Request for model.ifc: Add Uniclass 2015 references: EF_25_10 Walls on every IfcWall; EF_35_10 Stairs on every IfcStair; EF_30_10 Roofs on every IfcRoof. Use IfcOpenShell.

First a look at what the model holds.

```python
import ifcopenshell

model = ifcopenshell.open("model.ifc")
print(model.schema)
print("classifications:", [c.Name for c in model.by_type("IfcClassification")])
for ifc_class in ("IfcDoor", "IfcRoof", "IfcStair", "IfcWall", "IfcWindow"):
    print(ifc_class, len(model.by_type(ifc_class)))
```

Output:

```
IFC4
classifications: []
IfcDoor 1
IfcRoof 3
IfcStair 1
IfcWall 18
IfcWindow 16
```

```python
import ifcopenshell
import ifcopenshell.api.classification

model = ifcopenshell.open("model.ifc")

system = ifcopenshell.api.classification.add_classification(model, classification="Uniclass 2015")

codes = {
    "IfcWall": ("EF_25_10", "Walls"),
    "IfcStair": ("EF_35_10", "Stairs"),
    "IfcRoof": ("EF_30_10", "Roofs"),
}
for ifc_class, (code, name) in codes.items():
    products = model.by_type(ifc_class)
    ifcopenshell.api.classification.add_reference(
        model, products=products, classification=system, identification=code, name=name
    )
    print(code, len(products))

model.write("model_updated.ifc")
```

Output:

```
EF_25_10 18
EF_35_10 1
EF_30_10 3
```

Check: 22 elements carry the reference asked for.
